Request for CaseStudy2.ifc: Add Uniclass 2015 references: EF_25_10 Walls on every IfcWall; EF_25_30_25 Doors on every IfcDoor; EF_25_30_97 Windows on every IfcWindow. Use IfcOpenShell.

First a look at what the model holds.

```python
import ifcopenshell

model = ifcopenshell.open("CaseStudy2.ifc")
print(model.schema)
print("classifications:", [c.Name for c in model.by_type("IfcClassification")])
for ifc_class in ("IfcDoor", "IfcRoof", "IfcStair", "IfcWall", "IfcWindow"):
    print(ifc_class, len(model.by_type(ifc_class)))
```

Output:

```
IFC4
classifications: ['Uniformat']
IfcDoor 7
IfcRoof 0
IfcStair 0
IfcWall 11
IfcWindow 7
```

```python
import ifcopenshell
import ifcopenshell.api.classification

model = ifcopenshell.open("CaseStudy2.ifc")

system = ifcopenshell.api.classification.add_classification(model, classification="Uniclass 2015")

codes = {
    "IfcWall": ("EF_25_10", "Walls"),
    "IfcDoor": ("EF_25_30_25", "Doors"),
    "IfcWindow": ("EF_25_30_97", "Windows"),
}
for ifc_class, (code, name) in codes.items():
    products = model.by_type(ifc_class)
    ifcopenshell.api.classification.add_reference(
        model, products=products, classification=system, identification=code, name=name
    )
    print(code, len(products))

model.write("CaseStudy2-out.ifc")
```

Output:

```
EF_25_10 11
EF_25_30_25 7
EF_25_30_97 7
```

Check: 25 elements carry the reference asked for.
